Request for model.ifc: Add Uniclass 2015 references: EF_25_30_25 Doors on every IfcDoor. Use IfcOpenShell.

First a look at what the model holds.

```python
import ifcopenshell

model = ifcopenshell.open("model.ifc")
print(model.schema)
print("classifications:", [c.Name for c in model.by_type("IfcClassification")])
for ifc_class in ("IfcDoor", "IfcRoof", "IfcStair", "IfcWall", "IfcWindow"):
    print(ifc_class, len(model.by_type(ifc_class)))
```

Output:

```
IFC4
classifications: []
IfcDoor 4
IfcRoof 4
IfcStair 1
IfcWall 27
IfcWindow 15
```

```python
import ifcopenshell
import ifcopenshell.api.classification

model = ifcopenshell.open("model.ifc")

system = ifcopenshell.api.classification.add_classification(model, classification="Uniclass 2015")

codes = {
    "IfcDoor": ("EF_25_30_25", "Doors"),
}
for ifc_class, (code, name) in codes.items():
    products = model.by_type(ifc_class)
    ifcopenshell.api.classification.add_reference(
        model, products=products, classification=system, identification=code, name=name
    )
    print(code, len(products))

model.write("model-out.ifc")
```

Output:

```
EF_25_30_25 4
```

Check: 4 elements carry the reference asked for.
